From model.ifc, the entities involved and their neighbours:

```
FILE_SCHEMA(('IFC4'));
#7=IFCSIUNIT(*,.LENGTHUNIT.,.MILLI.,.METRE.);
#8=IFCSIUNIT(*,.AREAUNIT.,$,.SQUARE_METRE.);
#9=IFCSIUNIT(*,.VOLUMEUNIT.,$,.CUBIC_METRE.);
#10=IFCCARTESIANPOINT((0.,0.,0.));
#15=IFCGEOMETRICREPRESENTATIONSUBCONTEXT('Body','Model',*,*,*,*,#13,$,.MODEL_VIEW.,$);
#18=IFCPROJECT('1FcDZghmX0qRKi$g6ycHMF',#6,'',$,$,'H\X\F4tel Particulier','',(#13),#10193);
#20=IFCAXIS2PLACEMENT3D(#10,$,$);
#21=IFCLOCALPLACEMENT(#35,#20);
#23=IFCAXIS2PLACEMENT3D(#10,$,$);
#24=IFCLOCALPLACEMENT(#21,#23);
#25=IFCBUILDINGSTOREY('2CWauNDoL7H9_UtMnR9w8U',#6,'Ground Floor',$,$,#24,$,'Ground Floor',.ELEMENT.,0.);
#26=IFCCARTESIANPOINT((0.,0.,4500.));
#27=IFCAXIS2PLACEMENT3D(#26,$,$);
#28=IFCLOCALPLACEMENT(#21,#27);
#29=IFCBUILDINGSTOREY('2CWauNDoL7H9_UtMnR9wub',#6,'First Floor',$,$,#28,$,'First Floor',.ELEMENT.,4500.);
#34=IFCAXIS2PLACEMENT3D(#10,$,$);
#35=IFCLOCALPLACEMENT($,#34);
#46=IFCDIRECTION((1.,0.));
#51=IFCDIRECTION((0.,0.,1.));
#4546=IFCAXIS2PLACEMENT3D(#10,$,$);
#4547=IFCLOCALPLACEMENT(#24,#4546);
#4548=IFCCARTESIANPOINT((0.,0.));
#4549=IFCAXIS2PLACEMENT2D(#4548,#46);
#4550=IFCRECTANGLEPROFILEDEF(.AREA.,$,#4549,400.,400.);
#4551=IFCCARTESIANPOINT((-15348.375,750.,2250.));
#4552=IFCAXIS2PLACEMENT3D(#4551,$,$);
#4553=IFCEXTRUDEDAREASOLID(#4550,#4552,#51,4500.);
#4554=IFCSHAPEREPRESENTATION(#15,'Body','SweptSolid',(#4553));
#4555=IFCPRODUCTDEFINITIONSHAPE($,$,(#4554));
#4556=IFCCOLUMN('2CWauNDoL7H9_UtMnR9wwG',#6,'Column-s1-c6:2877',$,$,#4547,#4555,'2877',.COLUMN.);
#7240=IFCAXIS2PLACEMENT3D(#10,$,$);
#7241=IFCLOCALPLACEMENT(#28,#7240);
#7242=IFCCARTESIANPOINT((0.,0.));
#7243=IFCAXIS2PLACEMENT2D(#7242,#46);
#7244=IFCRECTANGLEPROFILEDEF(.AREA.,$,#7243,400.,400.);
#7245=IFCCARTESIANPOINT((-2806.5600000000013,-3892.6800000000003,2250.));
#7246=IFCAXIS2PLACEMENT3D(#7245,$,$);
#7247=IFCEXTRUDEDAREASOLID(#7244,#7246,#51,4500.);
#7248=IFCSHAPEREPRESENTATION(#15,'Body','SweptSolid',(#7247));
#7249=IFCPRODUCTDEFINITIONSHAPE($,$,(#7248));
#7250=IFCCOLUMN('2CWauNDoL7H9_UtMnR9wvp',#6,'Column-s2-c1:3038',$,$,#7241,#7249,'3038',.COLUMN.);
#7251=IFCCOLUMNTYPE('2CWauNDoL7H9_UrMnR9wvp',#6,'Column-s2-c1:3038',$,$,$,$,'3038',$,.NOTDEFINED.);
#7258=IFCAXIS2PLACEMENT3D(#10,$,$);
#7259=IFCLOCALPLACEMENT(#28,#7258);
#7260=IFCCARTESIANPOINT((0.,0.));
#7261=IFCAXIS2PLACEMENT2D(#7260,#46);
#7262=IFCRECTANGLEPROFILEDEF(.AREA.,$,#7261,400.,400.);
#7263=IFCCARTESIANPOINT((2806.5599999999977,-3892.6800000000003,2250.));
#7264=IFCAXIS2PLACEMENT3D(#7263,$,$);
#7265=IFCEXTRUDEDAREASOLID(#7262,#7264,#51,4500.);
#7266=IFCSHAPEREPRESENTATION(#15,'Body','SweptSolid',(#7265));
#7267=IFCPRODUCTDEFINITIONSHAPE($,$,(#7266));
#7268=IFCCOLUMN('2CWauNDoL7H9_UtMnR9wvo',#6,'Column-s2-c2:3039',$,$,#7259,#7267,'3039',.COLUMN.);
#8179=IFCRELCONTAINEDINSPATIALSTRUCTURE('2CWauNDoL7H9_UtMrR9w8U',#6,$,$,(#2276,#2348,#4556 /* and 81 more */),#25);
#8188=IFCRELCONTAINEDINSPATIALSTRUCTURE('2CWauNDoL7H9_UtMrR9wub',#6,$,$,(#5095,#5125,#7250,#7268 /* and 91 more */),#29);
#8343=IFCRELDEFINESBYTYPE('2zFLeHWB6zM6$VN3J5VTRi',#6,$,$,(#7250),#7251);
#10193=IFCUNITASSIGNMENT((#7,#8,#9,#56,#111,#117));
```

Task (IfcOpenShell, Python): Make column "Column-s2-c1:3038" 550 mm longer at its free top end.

```python
import ifcopenshell
import ifcopenshell.util.representation

model = ifcopenshell.open("model.ifc")

member = model.by_guid("2CWauNDoL7H9_UtMnR9wvp")
change = 550.0

# The extrusion runs towards the end named, so only its depth changes.
body = ifcopenshell.util.representation.get_representation(member, "Model", "Body")
solid = body.Items[0]
old_length = solid.Depth
solid.Depth += change

print(f"length {old_length:g} -> {solid.Depth:g}")

model.write("model-out.ifc")
```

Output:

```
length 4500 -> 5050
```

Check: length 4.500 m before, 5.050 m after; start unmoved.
